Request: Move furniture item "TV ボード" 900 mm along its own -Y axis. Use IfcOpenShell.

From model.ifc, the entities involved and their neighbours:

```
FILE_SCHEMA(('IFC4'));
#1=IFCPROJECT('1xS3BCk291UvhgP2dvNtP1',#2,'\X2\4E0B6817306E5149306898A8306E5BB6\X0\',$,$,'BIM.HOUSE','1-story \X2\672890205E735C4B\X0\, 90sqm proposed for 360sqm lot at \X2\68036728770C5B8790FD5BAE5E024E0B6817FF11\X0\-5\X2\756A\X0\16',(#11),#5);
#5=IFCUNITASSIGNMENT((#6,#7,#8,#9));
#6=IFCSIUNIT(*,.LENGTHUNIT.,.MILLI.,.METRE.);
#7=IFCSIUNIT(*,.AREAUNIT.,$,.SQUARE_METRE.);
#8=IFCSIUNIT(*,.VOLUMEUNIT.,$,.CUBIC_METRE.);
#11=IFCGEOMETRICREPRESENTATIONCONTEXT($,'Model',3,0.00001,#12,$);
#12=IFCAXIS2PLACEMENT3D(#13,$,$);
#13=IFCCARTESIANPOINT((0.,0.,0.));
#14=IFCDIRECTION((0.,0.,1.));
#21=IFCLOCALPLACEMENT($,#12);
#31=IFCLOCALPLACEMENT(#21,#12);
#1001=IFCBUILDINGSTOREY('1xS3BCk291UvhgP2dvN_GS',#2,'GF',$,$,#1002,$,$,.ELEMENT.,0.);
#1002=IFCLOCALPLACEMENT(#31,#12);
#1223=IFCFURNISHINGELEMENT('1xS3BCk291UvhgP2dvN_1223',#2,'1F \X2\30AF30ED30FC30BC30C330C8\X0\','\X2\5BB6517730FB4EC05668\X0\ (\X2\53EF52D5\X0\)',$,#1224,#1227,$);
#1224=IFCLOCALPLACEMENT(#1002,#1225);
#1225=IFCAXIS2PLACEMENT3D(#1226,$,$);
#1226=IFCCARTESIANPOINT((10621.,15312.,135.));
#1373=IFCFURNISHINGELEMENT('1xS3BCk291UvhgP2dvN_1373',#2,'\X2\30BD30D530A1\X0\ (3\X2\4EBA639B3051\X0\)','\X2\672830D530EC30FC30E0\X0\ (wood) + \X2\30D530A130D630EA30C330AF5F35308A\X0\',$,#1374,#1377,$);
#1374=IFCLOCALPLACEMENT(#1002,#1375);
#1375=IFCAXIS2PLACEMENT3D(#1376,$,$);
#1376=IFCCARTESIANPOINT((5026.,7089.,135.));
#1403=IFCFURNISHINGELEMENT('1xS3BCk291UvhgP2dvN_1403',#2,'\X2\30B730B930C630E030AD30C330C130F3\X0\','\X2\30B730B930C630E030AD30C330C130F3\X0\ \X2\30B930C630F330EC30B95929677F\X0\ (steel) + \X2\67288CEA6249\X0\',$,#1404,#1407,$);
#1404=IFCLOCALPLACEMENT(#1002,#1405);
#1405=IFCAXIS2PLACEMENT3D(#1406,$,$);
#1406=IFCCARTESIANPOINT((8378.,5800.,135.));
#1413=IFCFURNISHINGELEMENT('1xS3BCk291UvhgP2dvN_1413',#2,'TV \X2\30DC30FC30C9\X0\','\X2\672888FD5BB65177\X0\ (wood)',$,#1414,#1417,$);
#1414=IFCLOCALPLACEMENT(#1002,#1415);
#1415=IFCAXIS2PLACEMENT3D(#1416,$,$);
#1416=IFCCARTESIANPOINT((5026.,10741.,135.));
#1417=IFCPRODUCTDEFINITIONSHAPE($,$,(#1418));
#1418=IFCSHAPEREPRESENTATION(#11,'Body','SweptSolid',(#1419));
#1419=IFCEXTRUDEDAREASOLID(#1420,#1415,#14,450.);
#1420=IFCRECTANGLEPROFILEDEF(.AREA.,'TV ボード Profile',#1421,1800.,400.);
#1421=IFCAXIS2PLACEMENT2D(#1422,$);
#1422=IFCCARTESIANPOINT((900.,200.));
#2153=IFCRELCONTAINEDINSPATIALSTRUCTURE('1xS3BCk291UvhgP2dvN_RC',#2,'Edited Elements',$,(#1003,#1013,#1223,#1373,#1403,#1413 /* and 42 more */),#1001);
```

```python
import ifcopenshell
import ifcopenshell.api.geometry
import ifcopenshell.util.placement

model = ifcopenshell.open("model.ifc")

item = model.by_guid("1xS3BCk291UvhgP2dvN_1413")
matrix = ifcopenshell.util.placement.get_local_placement(item.ObjectPlacement)
matrix[:3, 3] -= matrix[:3, 1] * 900.0
ifcopenshell.api.geometry.edit_object_placement(model, product=item, matrix=matrix, is_si=False)

print(ifcopenshell.util.placement.get_local_placement(item.ObjectPlacement).round(3) + 0.0)

model.write("model_v2.ifc")
```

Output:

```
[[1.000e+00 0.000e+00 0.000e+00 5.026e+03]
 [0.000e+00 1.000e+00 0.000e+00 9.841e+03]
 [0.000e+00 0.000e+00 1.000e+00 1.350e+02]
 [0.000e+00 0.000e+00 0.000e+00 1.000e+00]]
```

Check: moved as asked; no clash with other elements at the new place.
